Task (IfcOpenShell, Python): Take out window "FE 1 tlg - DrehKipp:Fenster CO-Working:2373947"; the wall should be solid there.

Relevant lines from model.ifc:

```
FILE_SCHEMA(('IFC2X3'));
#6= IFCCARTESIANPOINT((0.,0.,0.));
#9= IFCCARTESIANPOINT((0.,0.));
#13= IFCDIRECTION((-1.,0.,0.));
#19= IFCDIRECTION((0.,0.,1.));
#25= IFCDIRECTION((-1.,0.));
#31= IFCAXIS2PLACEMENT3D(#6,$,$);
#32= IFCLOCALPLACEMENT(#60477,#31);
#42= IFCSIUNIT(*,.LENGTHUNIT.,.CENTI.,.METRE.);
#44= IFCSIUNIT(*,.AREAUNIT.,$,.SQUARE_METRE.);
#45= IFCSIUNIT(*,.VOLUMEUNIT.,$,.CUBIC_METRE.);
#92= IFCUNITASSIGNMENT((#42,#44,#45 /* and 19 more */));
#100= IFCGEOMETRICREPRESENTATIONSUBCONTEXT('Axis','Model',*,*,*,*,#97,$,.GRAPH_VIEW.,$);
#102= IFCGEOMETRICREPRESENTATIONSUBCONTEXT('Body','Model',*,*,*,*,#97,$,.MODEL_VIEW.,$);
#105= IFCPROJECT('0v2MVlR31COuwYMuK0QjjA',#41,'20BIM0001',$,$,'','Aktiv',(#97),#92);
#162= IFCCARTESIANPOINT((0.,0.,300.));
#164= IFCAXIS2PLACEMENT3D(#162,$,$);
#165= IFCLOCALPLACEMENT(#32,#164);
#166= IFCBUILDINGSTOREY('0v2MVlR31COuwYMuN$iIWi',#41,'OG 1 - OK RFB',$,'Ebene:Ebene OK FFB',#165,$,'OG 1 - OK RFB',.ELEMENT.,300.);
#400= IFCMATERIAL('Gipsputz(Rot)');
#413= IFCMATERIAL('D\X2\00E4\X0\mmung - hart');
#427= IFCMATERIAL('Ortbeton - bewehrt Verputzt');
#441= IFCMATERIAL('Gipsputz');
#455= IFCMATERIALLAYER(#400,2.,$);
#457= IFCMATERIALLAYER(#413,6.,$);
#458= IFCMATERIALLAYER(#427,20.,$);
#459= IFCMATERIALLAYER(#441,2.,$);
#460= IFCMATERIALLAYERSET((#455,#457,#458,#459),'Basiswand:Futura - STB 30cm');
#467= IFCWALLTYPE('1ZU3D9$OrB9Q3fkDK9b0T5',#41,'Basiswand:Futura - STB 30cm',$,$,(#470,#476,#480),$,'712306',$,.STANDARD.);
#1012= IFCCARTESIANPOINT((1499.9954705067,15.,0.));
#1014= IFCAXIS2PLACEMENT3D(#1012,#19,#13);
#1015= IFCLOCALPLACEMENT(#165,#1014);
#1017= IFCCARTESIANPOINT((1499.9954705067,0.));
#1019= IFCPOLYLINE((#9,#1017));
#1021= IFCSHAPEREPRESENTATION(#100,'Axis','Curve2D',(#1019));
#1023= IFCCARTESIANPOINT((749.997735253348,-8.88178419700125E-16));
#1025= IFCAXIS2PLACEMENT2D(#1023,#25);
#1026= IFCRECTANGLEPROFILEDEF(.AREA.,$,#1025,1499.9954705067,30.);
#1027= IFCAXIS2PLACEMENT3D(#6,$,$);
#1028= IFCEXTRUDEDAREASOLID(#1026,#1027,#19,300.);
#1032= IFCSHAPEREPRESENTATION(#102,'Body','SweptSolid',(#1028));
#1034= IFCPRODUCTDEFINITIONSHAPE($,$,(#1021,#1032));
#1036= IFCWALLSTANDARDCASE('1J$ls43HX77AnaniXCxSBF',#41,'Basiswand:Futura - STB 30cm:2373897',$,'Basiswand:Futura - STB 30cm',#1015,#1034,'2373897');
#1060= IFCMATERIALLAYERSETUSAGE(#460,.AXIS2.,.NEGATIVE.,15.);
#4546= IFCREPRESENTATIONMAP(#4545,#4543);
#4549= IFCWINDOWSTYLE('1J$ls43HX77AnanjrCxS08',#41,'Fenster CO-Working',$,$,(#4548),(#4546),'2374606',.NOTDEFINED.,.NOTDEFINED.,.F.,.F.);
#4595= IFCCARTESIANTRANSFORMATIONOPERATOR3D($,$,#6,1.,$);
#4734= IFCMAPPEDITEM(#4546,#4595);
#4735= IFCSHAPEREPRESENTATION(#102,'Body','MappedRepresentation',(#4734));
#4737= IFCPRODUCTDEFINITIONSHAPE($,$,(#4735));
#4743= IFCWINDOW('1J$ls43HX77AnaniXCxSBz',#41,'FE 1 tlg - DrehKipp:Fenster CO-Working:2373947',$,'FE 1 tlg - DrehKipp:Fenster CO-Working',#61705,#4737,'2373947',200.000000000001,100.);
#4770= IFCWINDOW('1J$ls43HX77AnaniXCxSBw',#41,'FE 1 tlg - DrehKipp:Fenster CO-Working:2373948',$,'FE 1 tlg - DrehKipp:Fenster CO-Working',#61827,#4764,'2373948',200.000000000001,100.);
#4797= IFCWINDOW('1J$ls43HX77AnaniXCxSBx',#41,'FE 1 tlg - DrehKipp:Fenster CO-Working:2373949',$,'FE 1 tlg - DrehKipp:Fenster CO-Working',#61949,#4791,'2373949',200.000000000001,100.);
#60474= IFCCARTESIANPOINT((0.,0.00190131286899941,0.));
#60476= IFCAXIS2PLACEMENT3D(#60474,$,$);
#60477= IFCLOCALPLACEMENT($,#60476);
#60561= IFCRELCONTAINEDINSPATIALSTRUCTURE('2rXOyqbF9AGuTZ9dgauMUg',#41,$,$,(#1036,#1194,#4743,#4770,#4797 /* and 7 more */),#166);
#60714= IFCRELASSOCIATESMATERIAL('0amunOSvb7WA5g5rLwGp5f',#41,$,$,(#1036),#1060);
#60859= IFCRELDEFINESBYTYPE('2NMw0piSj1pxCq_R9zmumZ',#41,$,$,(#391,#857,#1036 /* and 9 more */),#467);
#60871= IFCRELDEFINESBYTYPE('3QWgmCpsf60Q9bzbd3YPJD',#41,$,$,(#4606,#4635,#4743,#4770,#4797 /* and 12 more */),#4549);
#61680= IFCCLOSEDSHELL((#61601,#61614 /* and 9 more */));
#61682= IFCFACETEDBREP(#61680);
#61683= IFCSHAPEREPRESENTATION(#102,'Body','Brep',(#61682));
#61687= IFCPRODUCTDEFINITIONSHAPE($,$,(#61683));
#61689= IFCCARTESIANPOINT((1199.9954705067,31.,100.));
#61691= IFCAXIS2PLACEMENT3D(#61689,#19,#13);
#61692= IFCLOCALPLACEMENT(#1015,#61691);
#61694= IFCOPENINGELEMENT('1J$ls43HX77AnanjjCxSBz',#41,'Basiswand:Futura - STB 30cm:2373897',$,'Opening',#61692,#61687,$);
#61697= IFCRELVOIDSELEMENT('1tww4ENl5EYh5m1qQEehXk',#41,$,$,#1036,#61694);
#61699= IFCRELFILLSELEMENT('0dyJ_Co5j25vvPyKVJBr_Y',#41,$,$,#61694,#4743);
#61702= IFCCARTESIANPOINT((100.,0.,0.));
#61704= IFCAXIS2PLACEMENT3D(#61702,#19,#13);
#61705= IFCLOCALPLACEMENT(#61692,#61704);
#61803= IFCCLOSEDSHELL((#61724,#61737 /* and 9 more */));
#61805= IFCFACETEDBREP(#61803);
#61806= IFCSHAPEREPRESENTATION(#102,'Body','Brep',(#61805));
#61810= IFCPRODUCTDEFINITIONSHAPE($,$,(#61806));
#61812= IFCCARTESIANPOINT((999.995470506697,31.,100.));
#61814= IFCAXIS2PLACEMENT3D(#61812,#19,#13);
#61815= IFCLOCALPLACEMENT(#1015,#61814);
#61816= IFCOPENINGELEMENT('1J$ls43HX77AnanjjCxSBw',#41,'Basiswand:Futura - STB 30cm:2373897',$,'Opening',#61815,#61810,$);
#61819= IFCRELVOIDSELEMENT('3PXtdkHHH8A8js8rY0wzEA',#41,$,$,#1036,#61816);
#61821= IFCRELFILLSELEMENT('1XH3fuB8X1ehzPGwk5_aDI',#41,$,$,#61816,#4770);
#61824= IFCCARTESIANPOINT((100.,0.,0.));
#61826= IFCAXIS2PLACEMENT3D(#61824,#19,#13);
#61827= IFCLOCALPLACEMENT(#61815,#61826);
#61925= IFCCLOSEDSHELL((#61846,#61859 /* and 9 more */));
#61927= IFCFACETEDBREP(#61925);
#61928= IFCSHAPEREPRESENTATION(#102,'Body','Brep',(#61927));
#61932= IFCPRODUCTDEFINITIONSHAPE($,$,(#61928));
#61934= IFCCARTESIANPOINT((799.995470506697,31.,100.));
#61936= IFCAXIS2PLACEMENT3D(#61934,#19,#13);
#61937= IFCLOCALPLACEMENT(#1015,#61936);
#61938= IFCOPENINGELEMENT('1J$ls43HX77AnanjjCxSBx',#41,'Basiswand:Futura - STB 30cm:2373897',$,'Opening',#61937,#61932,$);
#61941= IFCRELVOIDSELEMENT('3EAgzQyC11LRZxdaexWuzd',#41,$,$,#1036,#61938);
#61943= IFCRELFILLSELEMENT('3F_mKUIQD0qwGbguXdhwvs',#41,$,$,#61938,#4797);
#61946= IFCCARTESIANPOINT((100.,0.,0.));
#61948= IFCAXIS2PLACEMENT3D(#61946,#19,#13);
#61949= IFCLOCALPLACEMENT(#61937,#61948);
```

```python
import ifcopenshell
import ifcopenshell.api.feature
import ifcopenshell.api.root
import ifcopenshell.geom
import ifcopenshell.util.shape

model = ifcopenshell.open("model.ifc")
settings = ifcopenshell.geom.settings()


def volume(element):
    """Net volume in cubic metres, openings subtracted."""
    shape = ifcopenshell.geom.create_shape(settings, element)
    return ifcopenshell.util.shape.get_volume(shape.geometry)


window = model.by_guid("1J$ls43HX77AnaniXCxSBz")
opening = window.FillsVoids[0].RelatingOpeningElement
wall = opening.VoidsElements[0].RelatingBuildingElement
before = volume(wall)

ifcopenshell.api.root.remove_product(model, product=window)
ifcopenshell.api.feature.remove_feature(model, feature=opening)

after = volume(wall)

print(f"wall volume {before:.3f} -> {after:.3f} m3")

model.write("model-out.ifc")
```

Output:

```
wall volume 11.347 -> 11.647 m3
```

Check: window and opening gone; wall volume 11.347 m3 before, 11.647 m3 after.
